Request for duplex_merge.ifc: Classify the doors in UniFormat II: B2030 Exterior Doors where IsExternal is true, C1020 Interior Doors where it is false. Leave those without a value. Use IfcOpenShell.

First a look at what the model holds.

```python
import ifcopenshell
import ifcopenshell.util.element

model = ifcopenshell.open("duplex_merge.ifc")
print(model.schema)
print("classifications:", [c.Name for c in model.by_type("IfcClassification")])
values = [ifcopenshell.util.element.get_pset(e, "Pset_DoorCommon", "IsExternal") for e in model.by_type("IfcDoor")]
for value in (True, False, None):
    print("IsExternal", value, values.count(value))
```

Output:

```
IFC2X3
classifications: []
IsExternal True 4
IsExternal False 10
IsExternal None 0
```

```python
import ifcopenshell
import ifcopenshell.api.classification
import ifcopenshell.util.element

model = ifcopenshell.open("duplex_merge.ifc")

# IFC2X3 requires Source and Edition and has no link from the project to the system.
system = model.create_entity("IfcClassification", Source="ASTM", Edition="E1557", Name="UniFormat II")

doors = model.by_type("IfcDoor")
external = {e: ifcopenshell.util.element.get_pset(e, "Pset_DoorCommon", "IsExternal") for e in doors}
for flag, code, name in ((True, "B2030", "Exterior Doors"), (False, "C1020", "Interior Doors")):
    products = [e for e in doors if external[e] is flag]
    ifcopenshell.api.classification.add_reference(
        model, products=products, classification=system, identification=code, name=name
    )
    print(code, len(products))

model.write("duplex_merge_updated.ifc")
```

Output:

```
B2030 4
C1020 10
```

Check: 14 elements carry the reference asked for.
